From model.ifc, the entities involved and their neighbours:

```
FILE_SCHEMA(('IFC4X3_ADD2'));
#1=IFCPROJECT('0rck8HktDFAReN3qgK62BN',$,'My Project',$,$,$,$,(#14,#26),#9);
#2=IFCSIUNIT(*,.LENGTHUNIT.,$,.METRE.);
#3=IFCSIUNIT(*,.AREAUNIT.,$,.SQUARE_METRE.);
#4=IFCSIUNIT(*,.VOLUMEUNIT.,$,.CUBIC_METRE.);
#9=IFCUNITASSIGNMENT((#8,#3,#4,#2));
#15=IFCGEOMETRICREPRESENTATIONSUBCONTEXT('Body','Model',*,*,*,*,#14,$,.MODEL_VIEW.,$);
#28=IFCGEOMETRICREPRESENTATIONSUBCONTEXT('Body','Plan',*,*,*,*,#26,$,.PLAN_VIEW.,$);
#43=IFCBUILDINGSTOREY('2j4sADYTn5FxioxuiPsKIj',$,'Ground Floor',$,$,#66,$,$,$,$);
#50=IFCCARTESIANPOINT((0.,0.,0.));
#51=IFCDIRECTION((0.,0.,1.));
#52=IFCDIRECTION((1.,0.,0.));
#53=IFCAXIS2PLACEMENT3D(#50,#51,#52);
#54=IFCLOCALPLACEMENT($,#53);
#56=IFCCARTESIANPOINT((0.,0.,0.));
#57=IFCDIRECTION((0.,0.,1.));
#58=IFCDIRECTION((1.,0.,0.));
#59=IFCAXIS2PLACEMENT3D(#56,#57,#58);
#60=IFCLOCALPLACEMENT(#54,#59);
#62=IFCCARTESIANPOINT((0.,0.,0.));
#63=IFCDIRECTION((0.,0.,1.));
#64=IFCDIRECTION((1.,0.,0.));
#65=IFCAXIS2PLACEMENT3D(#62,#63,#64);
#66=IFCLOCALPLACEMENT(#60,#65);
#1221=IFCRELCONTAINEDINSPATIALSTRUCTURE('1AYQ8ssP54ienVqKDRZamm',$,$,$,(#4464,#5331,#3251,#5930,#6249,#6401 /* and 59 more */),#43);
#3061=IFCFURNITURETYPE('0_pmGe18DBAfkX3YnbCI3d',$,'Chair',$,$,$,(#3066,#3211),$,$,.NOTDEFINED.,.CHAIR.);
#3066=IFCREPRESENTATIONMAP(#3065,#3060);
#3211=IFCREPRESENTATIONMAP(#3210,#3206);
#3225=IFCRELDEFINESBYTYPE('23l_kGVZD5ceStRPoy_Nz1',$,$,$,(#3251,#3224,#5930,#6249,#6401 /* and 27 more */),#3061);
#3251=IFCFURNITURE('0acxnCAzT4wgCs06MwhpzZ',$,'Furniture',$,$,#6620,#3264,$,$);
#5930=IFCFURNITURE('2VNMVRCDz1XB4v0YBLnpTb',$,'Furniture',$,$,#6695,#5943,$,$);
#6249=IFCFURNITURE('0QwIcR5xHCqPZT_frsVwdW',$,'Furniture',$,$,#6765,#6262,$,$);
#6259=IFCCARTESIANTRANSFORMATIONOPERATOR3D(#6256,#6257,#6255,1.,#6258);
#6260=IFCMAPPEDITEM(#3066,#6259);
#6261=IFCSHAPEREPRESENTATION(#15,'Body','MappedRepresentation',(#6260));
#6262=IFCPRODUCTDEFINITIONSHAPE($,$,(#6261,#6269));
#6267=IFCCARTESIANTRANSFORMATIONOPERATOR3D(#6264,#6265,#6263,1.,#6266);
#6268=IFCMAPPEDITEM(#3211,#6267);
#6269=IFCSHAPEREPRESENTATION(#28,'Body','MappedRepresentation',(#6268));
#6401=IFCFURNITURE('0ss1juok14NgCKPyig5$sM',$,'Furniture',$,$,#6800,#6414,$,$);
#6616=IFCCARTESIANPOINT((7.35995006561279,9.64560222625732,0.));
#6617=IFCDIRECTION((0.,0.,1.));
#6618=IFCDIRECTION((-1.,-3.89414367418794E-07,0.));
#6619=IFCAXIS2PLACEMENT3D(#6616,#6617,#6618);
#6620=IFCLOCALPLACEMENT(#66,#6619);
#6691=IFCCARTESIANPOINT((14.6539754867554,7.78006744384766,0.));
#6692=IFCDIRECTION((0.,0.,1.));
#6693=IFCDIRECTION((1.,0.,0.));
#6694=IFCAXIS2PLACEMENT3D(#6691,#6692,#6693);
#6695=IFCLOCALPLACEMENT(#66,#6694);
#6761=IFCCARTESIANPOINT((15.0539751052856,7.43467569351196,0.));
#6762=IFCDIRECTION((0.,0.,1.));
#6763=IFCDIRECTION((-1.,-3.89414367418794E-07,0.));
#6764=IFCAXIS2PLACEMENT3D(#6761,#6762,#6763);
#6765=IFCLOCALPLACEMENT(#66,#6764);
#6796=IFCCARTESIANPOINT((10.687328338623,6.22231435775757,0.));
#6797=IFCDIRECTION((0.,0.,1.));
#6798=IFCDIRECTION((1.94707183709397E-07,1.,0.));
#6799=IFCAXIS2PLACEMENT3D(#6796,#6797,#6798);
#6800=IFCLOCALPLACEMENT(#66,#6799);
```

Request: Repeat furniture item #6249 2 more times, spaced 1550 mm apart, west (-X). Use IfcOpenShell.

```python
import numpy as np
import ifcopenshell
import ifcopenshell.api.geometry
import ifcopenshell.api.root
import ifcopenshell.util.element
import ifcopenshell.util.placement
import ifcopenshell.util.unit

model = ifcopenshell.open("model.ifc")
unit_scale = ifcopenshell.util.unit.calculate_unit_scale(model)

source = model.by_guid("0QwIcR5xHCqPZT_frsVwdW")
base = ifcopenshell.util.placement.get_local_placement(source.ObjectPlacement)
step = np.array([-1.0, 0.0, 0.0]) * 1.55 / unit_scale

for i in range(1, 3):
    copy = ifcopenshell.api.root.copy_class(model, product=source)
    copy.Representation = ifcopenshell.util.element.copy_deep(
        model, source.Representation, exclude=["IfcGeometricRepresentationContext", "IfcRepresentationMap"]
    )
    matrix = base.copy()
    matrix[:3, 3] += i * step
    print("added at", matrix[:3, 3].round(3) + 0.0)
    ifcopenshell.api.geometry.edit_object_placement(model, product=copy, matrix=matrix, is_si=False)

model.write("model_updated.ifc")
```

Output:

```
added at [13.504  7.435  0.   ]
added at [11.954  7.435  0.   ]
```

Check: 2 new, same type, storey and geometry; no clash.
